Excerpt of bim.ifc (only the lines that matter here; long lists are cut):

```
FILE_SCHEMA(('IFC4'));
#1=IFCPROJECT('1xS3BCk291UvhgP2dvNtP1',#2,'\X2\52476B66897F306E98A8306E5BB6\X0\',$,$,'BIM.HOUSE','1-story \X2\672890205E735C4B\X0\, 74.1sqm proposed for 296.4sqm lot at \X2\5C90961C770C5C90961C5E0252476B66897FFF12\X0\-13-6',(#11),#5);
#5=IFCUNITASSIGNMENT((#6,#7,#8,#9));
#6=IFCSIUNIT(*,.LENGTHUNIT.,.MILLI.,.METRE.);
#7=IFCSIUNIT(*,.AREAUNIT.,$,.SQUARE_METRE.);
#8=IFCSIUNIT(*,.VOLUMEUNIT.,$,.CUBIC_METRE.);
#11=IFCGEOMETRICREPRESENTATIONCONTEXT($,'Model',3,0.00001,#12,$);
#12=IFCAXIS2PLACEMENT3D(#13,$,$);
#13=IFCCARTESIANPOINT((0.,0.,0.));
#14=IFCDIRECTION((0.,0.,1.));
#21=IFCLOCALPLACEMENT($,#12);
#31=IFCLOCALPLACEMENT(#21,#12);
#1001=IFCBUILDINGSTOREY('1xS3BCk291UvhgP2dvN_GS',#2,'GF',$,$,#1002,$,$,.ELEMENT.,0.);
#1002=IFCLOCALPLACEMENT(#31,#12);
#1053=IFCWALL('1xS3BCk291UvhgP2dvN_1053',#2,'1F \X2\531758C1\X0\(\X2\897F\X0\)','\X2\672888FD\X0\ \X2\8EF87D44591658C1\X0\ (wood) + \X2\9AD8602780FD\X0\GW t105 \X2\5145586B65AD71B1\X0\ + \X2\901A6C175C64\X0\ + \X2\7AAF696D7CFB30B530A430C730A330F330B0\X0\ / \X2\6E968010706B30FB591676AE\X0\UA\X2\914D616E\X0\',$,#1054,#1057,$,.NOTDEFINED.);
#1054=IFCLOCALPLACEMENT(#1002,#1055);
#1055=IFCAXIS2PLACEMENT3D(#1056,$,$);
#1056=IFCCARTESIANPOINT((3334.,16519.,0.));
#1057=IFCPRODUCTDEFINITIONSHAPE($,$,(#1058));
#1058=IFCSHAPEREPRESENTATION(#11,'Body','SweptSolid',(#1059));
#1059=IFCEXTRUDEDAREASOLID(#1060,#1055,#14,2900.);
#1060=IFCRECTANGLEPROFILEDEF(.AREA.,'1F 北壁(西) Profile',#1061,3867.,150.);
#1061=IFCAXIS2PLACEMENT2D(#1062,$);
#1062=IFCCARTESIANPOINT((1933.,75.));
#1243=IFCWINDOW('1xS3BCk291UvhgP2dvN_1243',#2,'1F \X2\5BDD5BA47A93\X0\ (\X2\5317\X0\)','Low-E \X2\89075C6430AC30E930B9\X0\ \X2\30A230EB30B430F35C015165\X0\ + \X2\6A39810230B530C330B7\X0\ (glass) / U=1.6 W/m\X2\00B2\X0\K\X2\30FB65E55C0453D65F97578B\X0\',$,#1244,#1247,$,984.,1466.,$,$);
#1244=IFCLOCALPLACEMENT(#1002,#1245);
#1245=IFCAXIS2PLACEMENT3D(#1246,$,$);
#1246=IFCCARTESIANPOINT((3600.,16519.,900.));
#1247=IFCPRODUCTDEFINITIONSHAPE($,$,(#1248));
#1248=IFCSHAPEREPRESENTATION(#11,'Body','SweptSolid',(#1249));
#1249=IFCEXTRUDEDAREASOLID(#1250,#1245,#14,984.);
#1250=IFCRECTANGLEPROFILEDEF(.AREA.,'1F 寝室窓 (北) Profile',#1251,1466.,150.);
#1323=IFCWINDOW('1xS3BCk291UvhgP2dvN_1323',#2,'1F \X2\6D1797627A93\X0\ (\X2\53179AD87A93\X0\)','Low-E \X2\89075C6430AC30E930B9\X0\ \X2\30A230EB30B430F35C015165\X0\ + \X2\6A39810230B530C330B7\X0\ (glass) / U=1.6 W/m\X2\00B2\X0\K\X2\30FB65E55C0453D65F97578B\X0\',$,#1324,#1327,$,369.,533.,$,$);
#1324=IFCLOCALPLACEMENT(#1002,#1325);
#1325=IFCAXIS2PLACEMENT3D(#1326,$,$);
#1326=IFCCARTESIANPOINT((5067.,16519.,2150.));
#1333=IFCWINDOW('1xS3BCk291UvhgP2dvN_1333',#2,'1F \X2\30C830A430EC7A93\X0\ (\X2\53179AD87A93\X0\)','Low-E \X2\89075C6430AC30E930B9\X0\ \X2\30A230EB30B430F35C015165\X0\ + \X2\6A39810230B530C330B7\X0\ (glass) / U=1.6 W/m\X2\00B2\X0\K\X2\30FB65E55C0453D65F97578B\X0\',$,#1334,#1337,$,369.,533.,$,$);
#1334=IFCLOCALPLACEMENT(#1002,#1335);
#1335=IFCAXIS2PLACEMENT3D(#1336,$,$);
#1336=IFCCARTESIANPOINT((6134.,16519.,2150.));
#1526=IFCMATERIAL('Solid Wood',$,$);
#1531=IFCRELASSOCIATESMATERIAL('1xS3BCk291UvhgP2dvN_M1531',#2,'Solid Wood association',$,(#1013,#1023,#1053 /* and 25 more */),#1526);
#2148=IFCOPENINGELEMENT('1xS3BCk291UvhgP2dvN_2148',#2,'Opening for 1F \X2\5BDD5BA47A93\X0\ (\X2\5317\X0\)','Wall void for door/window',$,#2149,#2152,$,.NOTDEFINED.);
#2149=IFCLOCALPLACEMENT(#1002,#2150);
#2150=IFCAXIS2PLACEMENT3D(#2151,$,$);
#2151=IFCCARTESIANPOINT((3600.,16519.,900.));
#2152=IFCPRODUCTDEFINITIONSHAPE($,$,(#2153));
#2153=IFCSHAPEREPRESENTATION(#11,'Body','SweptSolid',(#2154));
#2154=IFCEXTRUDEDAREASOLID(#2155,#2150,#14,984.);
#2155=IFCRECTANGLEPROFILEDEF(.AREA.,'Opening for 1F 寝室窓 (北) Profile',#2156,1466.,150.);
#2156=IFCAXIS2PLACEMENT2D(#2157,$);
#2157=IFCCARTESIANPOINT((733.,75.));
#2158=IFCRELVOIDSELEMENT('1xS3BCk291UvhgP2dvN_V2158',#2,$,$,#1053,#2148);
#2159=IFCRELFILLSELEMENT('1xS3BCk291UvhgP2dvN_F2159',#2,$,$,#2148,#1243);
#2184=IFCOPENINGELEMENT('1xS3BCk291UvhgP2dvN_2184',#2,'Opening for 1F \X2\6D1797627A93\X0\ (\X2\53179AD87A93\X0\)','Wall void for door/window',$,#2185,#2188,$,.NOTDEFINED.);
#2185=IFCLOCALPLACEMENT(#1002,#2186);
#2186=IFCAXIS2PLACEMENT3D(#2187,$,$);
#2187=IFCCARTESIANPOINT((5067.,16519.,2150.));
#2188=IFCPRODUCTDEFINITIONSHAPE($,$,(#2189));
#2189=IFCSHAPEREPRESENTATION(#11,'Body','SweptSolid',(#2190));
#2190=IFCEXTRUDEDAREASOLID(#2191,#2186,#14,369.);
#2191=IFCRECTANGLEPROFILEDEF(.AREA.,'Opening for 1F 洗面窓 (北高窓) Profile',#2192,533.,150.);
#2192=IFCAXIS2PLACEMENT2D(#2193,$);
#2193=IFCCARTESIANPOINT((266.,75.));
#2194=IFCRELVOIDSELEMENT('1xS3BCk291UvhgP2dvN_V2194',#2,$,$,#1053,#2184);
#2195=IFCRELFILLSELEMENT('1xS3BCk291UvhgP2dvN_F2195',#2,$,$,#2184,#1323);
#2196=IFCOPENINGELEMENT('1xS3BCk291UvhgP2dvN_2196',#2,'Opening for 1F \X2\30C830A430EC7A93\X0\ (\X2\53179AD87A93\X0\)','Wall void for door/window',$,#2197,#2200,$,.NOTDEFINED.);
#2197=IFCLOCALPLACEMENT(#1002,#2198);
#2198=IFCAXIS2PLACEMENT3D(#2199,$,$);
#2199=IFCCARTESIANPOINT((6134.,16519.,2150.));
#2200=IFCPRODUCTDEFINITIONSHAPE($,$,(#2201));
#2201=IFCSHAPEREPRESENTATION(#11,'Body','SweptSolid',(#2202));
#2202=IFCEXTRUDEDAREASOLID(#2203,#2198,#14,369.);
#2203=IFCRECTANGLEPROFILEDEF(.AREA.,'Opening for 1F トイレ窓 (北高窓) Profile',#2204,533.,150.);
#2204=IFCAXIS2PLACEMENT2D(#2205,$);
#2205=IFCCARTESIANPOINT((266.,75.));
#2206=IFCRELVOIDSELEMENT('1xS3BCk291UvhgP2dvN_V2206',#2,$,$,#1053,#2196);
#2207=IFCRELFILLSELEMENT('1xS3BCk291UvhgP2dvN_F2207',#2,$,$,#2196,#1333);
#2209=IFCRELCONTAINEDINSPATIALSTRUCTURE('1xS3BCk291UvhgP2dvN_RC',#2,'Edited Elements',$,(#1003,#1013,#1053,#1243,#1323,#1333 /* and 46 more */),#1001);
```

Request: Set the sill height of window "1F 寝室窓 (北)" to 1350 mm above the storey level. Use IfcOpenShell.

```python
import numpy as np
import ifcopenshell
import ifcopenshell.api.geometry
import ifcopenshell.geom
import ifcopenshell.util.element
import ifcopenshell.util.placement
import ifcopenshell.util.shape
import ifcopenshell.util.unit

model = ifcopenshell.open("bim.ifc")
unit_scale = ifcopenshell.util.unit.calculate_unit_scale(model)

window = model.by_guid("1xS3BCk291UvhgP2dvN_1243")
opening = window.FillsVoids[0].RelatingOpeningElement
storey = ifcopenshell.util.element.get_container(window, ifc_class="IfcBuildingStorey")
level = ifcopenshell.util.placement.get_local_placement(storey.ObjectPlacement)[2, 3]

# The opening's origin need not be at the sill, so measure its lowest point.
shape = ifcopenshell.geom.create_shape(ifcopenshell.geom.settings(), opening)
bottom = ifcopenshell.util.shape.get_shape_bottom_elevation(shape, shape.geometry) / unit_scale
dz = level + 1.35 / unit_scale - bottom

shift = np.array([0.0, 0.0, dz])
# The window is not placed relative to its opening, so move both.
for product in (opening, window):
    matrix = ifcopenshell.util.placement.get_local_placement(product.ObjectPlacement)
    matrix[:3, 3] += shift
    ifcopenshell.api.geometry.edit_object_placement(model, product=product, matrix=matrix, is_si=False)

print(f"moved by {dz * unit_scale:+.3f} m")

model.write("bim_edited.ifc")
```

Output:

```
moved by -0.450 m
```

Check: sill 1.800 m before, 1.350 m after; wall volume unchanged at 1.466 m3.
